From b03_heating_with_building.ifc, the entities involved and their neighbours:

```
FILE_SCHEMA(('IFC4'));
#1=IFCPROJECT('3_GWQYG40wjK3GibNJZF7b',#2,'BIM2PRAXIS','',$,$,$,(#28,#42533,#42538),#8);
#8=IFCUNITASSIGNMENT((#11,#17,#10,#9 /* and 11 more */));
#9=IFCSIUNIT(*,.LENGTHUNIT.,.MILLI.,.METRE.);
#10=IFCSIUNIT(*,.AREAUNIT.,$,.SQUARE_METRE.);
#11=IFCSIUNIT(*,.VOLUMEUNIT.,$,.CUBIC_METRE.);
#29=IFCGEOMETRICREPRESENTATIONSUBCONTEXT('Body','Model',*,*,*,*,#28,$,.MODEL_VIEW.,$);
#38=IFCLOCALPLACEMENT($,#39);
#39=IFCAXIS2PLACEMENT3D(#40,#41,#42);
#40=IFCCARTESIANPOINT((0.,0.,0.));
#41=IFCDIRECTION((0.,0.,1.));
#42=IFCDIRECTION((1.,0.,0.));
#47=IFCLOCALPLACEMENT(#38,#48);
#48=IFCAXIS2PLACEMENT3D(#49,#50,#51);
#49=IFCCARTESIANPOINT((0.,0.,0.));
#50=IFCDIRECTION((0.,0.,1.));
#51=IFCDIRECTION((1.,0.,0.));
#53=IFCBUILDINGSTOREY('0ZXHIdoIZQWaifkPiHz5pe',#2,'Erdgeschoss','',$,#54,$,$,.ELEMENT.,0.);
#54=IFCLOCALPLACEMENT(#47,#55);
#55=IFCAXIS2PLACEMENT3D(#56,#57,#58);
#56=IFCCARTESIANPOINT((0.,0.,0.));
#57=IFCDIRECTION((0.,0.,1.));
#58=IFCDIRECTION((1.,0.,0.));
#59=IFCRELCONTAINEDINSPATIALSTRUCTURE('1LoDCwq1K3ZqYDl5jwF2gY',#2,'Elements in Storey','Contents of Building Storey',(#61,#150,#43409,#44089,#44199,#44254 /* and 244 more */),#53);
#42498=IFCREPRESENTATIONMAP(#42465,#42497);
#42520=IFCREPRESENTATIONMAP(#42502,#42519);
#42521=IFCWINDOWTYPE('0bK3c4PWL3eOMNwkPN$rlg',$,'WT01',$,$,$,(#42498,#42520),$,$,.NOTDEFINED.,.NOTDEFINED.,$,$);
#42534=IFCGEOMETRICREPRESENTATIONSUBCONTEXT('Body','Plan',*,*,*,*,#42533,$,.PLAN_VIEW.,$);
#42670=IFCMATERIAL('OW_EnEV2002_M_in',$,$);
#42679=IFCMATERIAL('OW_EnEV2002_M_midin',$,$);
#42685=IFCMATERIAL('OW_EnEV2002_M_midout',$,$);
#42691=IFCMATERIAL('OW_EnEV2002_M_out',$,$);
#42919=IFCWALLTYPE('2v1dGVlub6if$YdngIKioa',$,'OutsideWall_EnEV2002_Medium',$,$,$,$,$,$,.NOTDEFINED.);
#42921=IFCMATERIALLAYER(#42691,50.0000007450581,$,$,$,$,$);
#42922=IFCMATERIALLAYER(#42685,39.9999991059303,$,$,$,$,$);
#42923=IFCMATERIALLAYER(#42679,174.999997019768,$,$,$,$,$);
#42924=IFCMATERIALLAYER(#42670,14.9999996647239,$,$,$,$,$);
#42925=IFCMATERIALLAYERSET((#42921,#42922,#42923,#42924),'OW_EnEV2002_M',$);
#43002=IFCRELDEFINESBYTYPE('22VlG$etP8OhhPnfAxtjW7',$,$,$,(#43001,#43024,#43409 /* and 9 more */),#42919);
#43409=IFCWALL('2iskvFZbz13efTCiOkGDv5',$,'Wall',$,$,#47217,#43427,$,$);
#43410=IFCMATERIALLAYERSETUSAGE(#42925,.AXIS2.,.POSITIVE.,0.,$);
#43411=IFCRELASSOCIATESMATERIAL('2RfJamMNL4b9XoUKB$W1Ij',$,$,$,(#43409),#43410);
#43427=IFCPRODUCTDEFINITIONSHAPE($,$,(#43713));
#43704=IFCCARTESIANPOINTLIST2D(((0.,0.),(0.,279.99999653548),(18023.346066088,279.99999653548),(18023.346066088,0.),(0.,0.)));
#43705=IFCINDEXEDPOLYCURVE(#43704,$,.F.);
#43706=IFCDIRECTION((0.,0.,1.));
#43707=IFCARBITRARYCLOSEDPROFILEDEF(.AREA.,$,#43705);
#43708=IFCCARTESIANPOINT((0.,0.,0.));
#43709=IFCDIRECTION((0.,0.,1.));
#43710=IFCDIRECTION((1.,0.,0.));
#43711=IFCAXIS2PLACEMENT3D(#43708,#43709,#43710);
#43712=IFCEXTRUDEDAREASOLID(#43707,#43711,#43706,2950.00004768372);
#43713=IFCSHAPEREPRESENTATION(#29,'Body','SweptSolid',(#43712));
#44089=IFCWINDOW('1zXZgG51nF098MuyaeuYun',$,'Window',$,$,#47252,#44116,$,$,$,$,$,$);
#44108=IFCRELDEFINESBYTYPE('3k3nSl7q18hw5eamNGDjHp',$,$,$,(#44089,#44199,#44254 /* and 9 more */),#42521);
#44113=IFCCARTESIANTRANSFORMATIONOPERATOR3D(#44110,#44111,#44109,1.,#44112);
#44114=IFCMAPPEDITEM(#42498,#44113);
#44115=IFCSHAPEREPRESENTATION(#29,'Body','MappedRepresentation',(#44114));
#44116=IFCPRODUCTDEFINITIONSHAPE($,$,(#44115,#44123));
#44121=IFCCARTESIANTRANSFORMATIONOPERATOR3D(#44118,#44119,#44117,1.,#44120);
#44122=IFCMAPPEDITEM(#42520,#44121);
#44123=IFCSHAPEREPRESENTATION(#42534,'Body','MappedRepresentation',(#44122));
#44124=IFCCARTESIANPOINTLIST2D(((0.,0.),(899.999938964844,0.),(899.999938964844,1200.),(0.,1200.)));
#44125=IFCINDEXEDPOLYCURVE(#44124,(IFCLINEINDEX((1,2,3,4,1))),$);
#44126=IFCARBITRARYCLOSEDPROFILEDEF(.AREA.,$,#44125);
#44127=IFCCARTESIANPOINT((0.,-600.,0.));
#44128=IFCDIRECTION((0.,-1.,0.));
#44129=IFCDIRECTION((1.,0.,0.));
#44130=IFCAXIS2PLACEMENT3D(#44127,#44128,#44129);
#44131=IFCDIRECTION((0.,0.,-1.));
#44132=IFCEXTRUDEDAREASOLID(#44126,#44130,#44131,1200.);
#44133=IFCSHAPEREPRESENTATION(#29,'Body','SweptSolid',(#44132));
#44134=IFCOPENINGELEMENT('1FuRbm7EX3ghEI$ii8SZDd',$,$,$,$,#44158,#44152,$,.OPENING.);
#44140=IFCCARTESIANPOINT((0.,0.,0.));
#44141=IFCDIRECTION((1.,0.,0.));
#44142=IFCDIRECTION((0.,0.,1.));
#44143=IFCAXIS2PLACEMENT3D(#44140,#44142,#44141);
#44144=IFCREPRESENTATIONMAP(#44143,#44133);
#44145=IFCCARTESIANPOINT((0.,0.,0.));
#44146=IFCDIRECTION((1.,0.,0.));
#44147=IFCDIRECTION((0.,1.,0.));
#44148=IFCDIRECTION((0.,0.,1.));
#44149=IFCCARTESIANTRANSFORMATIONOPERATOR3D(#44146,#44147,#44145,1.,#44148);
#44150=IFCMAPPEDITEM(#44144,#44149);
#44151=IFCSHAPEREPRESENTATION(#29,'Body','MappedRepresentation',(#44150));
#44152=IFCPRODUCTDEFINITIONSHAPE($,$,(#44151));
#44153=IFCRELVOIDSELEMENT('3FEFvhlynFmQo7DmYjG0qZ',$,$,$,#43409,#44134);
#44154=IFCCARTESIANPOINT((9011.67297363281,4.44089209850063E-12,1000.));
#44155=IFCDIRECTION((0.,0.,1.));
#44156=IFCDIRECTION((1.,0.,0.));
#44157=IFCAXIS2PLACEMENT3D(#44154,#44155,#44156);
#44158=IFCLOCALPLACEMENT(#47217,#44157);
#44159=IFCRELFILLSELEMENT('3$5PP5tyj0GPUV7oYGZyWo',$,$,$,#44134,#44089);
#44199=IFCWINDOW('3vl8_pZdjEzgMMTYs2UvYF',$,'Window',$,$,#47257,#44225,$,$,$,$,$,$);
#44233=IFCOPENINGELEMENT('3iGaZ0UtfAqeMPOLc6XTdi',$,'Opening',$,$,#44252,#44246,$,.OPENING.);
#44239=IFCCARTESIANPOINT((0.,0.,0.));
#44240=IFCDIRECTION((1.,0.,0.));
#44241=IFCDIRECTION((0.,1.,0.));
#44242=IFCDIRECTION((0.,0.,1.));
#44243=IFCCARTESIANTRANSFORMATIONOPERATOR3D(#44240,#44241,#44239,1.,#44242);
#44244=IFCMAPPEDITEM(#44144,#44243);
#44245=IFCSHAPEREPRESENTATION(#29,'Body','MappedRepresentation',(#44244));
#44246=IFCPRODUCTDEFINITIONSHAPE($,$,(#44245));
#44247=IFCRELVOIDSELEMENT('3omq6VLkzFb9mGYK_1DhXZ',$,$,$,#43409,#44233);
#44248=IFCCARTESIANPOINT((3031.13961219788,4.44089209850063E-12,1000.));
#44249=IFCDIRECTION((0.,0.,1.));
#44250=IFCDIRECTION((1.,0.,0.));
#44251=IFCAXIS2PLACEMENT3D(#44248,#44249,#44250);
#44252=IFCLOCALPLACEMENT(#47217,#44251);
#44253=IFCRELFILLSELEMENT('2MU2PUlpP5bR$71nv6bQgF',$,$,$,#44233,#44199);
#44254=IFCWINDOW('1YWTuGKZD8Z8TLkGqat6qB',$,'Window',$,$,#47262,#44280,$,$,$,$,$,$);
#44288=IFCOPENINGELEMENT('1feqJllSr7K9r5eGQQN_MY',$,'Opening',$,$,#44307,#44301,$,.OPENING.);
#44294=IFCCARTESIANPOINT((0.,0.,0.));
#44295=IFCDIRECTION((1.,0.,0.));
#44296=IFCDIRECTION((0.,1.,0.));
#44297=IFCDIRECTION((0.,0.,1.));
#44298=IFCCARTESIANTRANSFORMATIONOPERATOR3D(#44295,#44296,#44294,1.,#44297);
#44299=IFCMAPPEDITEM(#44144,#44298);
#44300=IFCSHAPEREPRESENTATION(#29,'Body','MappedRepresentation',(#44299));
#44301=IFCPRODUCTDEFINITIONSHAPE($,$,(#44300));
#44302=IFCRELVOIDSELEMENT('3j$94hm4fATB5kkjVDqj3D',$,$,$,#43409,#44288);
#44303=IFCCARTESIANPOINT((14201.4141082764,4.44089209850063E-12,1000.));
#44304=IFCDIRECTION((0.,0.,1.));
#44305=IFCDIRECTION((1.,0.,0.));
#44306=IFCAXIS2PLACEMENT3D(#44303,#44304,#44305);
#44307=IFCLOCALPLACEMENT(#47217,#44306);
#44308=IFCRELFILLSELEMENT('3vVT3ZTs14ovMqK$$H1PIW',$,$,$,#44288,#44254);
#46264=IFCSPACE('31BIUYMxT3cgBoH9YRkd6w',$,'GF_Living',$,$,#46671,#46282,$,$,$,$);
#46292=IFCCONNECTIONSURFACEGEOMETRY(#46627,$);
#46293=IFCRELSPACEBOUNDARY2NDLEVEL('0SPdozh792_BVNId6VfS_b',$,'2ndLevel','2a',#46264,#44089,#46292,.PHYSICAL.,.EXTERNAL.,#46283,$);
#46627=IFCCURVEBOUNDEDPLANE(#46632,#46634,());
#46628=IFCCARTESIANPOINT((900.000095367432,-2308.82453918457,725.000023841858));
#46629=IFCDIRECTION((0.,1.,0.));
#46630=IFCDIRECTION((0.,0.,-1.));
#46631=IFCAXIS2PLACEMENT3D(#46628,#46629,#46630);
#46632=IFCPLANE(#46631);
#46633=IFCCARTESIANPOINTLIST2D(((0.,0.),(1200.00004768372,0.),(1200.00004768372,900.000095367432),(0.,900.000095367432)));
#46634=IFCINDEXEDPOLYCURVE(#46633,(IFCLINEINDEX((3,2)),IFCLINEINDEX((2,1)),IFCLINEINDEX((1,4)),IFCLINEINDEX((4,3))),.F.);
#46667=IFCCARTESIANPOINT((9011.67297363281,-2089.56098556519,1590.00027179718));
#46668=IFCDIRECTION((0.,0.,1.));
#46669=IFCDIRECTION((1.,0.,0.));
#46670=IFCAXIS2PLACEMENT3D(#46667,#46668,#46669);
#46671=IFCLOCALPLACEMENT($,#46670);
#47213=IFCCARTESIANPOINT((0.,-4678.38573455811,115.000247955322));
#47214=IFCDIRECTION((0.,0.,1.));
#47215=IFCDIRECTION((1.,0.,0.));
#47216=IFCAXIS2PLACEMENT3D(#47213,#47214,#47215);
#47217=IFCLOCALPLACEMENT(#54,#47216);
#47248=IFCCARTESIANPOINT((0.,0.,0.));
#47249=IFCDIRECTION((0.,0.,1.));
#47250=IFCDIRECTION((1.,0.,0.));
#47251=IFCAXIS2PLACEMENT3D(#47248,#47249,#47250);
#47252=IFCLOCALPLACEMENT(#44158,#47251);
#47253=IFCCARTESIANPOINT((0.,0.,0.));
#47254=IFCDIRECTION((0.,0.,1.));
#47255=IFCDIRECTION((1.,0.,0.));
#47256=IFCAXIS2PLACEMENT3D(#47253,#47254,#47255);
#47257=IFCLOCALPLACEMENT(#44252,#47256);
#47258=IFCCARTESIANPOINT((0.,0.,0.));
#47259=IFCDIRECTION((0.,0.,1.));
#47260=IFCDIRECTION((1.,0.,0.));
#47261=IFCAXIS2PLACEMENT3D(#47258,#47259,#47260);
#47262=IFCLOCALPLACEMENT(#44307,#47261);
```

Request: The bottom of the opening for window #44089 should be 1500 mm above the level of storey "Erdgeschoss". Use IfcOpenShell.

```python
import numpy as np
import ifcopenshell
import ifcopenshell.api.geometry
import ifcopenshell.geom
import ifcopenshell.util.element
import ifcopenshell.util.placement
import ifcopenshell.util.shape
import ifcopenshell.util.unit

model = ifcopenshell.open("b03_heating_with_building.ifc")
unit_scale = ifcopenshell.util.unit.calculate_unit_scale(model)

window = model.by_guid("1zXZgG51nF098MuyaeuYun")
opening = window.FillsVoids[0].RelatingOpeningElement
storey = ifcopenshell.util.element.get_container(window, ifc_class="IfcBuildingStorey")
level = ifcopenshell.util.placement.get_local_placement(storey.ObjectPlacement)[2, 3]

# The opening's origin need not be at the sill, so measure its lowest point.
shape = ifcopenshell.geom.create_shape(ifcopenshell.geom.settings(), opening)
bottom = ifcopenshell.util.shape.get_shape_bottom_elevation(shape, shape.geometry) / unit_scale
dz = level + 1.5 / unit_scale - bottom

shift = np.array([0.0, 0.0, dz])
# The window is placed relative to its opening, so it follows when the opening moves.
matrix = ifcopenshell.util.placement.get_local_placement(opening.ObjectPlacement)
matrix[:3, 3] += shift
ifcopenshell.api.geometry.edit_object_placement(
    model, product=opening, matrix=matrix, is_si=False, should_transform_children=True
)

# Space boundary surfaces are stored in each space's coordinates; move them too.
for rel in window.ProvidesBoundaries:
    if not rel.ConnectionGeometry:
        continue
    surface = rel.ConnectionGeometry.SurfaceOnRelatingElement.BasisSurface
    space_matrix = ifcopenshell.util.placement.get_local_placement(rel.RelatingSpace.ObjectPlacement)
    point = np.array(surface.Position.Location.Coordinates) + space_matrix[:3, :3].T @ shift
    surface.Position = model.createIfcAxis2Placement3D(
        model.createIfcCartesianPoint(point.tolist()), surface.Position.Axis, surface.Position.RefDirection
    )

print(f"moved by {dz * unit_scale:+.3f} m")

model.write("b03_heating_with_building_updated.ifc")
```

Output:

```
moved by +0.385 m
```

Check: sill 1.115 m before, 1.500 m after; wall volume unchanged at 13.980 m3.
